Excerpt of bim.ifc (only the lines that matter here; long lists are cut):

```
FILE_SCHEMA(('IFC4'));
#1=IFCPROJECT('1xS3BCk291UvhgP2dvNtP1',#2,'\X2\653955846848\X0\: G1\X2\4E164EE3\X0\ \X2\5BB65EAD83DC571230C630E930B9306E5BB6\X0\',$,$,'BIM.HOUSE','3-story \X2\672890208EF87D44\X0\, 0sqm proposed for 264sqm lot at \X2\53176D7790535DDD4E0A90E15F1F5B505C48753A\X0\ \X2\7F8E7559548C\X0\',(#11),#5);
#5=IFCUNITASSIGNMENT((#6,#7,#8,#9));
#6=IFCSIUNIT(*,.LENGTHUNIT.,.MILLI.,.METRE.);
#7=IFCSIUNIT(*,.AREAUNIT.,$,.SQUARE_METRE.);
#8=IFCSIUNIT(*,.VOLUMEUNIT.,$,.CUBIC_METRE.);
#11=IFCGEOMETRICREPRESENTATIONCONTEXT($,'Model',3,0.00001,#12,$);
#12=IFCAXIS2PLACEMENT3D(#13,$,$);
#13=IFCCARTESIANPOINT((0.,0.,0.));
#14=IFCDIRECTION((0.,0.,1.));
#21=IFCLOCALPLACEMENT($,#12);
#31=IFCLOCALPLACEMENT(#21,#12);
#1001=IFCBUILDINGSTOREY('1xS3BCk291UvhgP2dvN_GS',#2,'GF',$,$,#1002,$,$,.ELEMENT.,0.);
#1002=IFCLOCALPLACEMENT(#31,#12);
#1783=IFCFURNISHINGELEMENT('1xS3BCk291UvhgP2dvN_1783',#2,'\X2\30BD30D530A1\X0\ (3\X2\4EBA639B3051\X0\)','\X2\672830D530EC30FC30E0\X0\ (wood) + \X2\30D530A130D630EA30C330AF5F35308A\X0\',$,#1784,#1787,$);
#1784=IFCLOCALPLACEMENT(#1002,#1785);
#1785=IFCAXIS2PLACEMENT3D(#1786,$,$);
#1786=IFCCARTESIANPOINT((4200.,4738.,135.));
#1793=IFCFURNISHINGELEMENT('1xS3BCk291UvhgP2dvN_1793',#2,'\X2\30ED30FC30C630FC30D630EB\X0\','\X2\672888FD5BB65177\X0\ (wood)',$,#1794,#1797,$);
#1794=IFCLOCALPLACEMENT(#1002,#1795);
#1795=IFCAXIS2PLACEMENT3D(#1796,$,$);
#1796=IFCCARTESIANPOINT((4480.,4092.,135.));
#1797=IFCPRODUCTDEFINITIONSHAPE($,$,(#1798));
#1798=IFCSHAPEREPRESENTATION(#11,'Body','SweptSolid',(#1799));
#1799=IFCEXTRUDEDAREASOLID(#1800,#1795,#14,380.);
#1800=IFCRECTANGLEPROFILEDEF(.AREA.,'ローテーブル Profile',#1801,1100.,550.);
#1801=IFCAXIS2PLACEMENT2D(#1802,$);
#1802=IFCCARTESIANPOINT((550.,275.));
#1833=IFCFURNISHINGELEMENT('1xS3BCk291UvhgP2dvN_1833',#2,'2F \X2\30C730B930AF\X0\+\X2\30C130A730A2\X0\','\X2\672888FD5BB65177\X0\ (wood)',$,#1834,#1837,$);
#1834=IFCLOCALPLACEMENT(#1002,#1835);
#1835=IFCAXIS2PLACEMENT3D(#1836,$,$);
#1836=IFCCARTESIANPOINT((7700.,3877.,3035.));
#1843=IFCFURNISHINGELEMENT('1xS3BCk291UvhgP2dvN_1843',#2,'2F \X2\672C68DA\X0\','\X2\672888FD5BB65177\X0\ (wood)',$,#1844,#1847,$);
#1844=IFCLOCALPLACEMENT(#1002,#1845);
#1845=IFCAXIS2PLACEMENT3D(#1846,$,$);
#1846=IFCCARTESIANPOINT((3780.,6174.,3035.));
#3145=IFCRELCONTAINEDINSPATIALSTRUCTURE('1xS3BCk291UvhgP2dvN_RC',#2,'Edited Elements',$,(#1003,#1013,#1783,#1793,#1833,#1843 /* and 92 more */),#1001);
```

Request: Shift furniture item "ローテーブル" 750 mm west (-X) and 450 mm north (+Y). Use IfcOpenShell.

```python
import ifcopenshell
import ifcopenshell.api.geometry
import ifcopenshell.util.placement
import ifcopenshell.util.unit

model = ifcopenshell.open("bim.ifc")
unit_scale = ifcopenshell.util.unit.calculate_unit_scale(model)

item = model.by_guid("1xS3BCk291UvhgP2dvN_1793")
matrix = ifcopenshell.util.placement.get_local_placement(item.ObjectPlacement)
matrix[0, 3] -= 0.75 / unit_scale
matrix[1, 3] += 0.45 / unit_scale
ifcopenshell.api.geometry.edit_object_placement(model, product=item, matrix=matrix, is_si=False)

print(ifcopenshell.util.placement.get_local_placement(item.ObjectPlacement).round(3) + 0.0)

model.write("bim_updated.ifc")
```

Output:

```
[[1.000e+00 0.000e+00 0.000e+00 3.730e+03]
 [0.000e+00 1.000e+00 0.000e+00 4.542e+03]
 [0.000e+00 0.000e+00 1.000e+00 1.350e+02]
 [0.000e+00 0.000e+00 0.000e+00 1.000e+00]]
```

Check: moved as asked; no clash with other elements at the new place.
